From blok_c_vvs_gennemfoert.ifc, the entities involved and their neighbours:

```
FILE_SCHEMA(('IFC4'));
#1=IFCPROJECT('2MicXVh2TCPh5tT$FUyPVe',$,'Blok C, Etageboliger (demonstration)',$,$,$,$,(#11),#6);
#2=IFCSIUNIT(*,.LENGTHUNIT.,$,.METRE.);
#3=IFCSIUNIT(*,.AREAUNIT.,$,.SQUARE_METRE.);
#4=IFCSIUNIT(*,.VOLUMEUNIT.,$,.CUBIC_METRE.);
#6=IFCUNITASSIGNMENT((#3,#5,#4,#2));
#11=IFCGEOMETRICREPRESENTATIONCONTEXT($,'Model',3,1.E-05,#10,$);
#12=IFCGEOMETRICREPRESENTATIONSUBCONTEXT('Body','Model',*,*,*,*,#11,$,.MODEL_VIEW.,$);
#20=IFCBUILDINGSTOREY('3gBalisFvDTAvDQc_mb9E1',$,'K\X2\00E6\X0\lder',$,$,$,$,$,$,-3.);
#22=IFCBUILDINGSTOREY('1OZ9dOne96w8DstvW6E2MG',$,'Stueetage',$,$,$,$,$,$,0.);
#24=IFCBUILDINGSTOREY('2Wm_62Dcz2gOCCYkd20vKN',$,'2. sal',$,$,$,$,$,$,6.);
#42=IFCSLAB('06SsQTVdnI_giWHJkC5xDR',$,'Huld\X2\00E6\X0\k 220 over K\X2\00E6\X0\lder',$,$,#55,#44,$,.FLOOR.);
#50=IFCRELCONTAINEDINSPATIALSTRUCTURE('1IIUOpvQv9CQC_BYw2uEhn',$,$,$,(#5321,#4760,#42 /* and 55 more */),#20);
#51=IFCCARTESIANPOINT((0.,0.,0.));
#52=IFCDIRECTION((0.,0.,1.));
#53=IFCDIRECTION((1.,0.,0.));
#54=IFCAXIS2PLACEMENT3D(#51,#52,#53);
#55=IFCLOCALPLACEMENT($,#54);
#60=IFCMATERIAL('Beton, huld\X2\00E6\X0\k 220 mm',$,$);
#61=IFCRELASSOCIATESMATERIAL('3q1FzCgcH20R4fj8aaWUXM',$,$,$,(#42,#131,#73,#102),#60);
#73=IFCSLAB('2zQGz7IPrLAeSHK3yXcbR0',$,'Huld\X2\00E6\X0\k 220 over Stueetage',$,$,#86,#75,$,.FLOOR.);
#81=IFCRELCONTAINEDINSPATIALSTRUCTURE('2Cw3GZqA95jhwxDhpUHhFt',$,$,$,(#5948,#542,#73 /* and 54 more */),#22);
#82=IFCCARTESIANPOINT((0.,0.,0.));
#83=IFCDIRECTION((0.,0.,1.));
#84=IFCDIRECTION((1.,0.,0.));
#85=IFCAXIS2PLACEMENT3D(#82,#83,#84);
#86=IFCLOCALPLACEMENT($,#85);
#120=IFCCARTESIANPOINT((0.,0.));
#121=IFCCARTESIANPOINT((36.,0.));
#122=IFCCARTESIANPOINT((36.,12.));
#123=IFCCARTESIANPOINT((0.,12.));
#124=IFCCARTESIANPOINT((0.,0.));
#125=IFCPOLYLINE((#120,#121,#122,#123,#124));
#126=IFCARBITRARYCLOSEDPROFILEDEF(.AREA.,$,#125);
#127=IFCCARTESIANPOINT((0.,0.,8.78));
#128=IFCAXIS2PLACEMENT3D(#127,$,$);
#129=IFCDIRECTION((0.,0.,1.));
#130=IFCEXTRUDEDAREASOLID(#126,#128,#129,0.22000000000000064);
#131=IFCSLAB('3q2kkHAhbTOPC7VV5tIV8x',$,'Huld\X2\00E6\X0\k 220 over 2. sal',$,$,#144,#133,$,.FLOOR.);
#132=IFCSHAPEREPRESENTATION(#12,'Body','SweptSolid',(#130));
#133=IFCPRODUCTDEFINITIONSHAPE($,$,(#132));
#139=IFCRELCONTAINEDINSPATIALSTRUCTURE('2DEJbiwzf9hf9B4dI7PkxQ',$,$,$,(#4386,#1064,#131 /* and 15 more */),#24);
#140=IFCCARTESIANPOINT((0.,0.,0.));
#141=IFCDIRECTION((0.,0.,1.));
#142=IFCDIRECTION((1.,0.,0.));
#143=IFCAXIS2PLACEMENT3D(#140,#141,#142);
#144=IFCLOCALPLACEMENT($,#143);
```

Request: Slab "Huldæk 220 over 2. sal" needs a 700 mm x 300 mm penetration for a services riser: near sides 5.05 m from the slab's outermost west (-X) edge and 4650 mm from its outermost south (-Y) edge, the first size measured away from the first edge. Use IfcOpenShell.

```python
import numpy as np
import ifcopenshell
import ifcopenshell.api.feature
import ifcopenshell.api.geometry
import ifcopenshell.api.root
import ifcopenshell.geom
import ifcopenshell.util.placement
import ifcopenshell.util.representation
import ifcopenshell.util.shape
import ifcopenshell.util.unit

model = ifcopenshell.open("blok_c_vvs_gennemfoert.ifc")
unit_scale = ifcopenshell.util.unit.calculate_unit_scale(model)
settings = ifcopenshell.geom.settings()


def volume(element):
    """Net volume in cubic metres, openings subtracted."""
    shape = ifcopenshell.geom.create_shape(settings, element)
    return ifcopenshell.util.shape.get_volume(shape.geometry)


slab = model.by_guid("3q2kkHAhbTOPC7VV5tIV8x")
before = volume(slab)

# Extent in the slab's own axes, in metres. The edges named are its -X and -Y sides.
slab_shape = ifcopenshell.geom.create_shape(settings, slab)
vertices = ifcopenshell.util.shape.get_vertices(slab_shape.geometry)
x_min, y_min, bottom = vertices.min(axis=0)
top = vertices[:, 2].max()

opening = ifcopenshell.api.root.create_entity(model, ifc_class="IfcOpeningElement", name="Services riser opening", predefined_type="OPENING")
context = ifcopenshell.util.representation.get_context(model, "Model", "Body", "MODEL_VIEW")
width, depth = 0.7, 0.3
outline = [(0.0, 0.0), (width, 0.0), (width, depth), (0.0, depth), (0.0, 0.0)]
# Overshoot both faces by 50 mm so the cut is clean.
shape = ifcopenshell.api.geometry.add_slab_representation(
    model, context=context, depth=top - bottom + 0.1, polyline=outline
)
ifcopenshell.api.geometry.assign_representation(model, product=opening, representation=shape)

matrix = ifcopenshell.util.placement.get_local_placement(slab.ObjectPlacement)
matrix[:, 3] = matrix @ np.append(np.array([x_min + 5.05, y_min + 4.65, bottom - 0.05]) / unit_scale, 1.0)
ifcopenshell.api.geometry.edit_object_placement(model, product=opening, matrix=matrix, is_si=False)
ifcopenshell.api.feature.add_feature(model, feature=opening, element=slab)

after = volume(slab)

print(f"slab volume {before:.3f} -> {after:.3f} m3")

model.write("blok_c_vvs_gennemfoert_updated.ifc")
```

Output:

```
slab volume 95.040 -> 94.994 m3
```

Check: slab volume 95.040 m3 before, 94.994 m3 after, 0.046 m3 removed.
